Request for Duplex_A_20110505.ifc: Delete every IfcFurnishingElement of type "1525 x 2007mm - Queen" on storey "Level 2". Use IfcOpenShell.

First a look at what the model holds.

```python
import ifcopenshell
import ifcopenshell.util.element

model = ifcopenshell.open("Duplex_A_20110505.ifc")
print(model.schema)
storey = next(s for s in model.by_type("IfcBuildingStorey") if s.Name == "Level 2")
furniture = [e for e in ifcopenshell.util.element.get_decomposition(storey) if e.is_a("IfcFurnishingElement")]
seen = {}
for e in furniture:
    element_type = ifcopenshell.util.element.get_type(e)
    name = element_type.Name if element_type not in (None, e) else None
    seen[name] = seen.get(name, 0) + 1
for name, count in sorted(seen.items(), key=str):
    print(count, "x", name)
```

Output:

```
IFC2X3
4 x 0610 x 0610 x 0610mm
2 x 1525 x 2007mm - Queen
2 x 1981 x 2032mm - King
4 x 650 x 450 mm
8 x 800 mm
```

```python
import ifcopenshell
import ifcopenshell.api.root
import ifcopenshell.util.element

model = ifcopenshell.open("Duplex_A_20110505.ifc")

storey = next(s for s in model.by_type("IfcBuildingStorey") if s.Name == "Level 2")
furniture = [e for e in ifcopenshell.util.element.get_decomposition(storey) if e.is_a("IfcFurnishingElement")]
targets = [e for e in furniture if (t := ifcopenshell.util.element.get_type(e)) not in (None, e) and t.Name == "1525 x 2007mm - Queen"]

for e in targets:
    ifcopenshell.api.root.remove_product(model, product=e)
print(len(targets), "removed")

model.write("Duplex_A_20110505_rev.ifc")
```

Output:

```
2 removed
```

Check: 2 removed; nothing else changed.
